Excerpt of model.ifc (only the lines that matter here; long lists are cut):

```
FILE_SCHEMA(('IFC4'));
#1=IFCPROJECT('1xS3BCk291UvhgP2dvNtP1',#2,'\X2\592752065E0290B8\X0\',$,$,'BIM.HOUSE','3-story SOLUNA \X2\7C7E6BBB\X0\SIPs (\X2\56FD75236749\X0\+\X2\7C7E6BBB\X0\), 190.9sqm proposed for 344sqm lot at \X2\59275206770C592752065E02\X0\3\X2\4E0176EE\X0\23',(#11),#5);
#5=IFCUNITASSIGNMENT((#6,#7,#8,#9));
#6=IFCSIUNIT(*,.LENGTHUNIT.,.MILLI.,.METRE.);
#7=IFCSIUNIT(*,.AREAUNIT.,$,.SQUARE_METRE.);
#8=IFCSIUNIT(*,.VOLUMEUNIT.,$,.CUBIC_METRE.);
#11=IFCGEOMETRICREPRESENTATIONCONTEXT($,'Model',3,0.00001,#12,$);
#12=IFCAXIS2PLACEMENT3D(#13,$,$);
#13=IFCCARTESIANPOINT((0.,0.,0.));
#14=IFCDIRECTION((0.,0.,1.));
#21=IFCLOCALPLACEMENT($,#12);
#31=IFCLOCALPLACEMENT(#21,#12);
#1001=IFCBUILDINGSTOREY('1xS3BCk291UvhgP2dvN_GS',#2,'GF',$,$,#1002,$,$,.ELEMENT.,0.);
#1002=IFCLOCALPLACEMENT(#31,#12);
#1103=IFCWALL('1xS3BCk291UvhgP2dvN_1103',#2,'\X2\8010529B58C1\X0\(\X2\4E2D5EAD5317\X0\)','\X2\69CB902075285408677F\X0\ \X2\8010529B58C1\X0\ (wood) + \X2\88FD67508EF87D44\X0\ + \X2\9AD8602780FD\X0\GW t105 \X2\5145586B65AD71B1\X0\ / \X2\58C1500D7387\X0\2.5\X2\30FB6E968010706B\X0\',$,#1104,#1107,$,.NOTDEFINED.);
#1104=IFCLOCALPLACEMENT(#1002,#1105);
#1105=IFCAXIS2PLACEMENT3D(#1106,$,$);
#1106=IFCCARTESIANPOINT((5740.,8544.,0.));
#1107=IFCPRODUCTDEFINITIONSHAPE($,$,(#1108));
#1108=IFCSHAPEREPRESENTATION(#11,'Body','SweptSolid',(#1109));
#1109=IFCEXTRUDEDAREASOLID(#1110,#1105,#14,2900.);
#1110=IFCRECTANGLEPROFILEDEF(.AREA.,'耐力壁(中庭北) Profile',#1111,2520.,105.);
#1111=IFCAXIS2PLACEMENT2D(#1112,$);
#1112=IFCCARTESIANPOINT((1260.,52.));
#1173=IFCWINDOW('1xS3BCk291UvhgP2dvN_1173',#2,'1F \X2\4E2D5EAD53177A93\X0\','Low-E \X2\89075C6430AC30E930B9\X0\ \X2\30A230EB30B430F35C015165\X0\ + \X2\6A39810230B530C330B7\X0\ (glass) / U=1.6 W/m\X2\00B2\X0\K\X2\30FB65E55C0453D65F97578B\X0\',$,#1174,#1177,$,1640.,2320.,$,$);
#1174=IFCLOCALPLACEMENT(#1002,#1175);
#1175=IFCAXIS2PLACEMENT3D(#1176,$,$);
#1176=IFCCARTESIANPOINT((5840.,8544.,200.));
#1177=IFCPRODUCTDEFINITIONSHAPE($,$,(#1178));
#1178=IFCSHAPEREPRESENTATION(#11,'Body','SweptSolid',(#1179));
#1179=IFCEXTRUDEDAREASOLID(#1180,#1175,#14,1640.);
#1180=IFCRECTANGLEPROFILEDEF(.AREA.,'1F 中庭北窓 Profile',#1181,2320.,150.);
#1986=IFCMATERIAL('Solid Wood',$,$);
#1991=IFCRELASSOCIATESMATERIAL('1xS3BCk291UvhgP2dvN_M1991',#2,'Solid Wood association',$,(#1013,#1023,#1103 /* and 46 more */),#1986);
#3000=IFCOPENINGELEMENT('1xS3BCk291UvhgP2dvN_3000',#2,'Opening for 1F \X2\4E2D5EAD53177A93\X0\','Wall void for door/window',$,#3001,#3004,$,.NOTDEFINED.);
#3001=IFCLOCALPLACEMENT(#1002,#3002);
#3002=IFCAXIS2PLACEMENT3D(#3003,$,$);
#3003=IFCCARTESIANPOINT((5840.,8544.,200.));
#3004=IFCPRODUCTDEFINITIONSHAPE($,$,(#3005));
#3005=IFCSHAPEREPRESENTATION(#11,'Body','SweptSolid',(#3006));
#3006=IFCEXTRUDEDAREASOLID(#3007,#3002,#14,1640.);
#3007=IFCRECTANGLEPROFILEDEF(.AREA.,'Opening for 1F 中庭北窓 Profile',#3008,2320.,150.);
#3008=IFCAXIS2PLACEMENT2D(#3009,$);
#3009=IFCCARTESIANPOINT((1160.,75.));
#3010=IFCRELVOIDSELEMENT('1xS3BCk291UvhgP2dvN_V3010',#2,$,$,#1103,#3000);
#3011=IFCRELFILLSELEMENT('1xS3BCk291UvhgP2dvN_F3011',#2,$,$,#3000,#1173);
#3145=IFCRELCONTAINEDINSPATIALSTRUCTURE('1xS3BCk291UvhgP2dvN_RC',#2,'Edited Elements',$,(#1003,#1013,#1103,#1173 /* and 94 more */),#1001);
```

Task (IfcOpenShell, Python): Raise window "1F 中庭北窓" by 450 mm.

```python
import numpy as np
import ifcopenshell
import ifcopenshell.api.geometry
import ifcopenshell.util.placement
import ifcopenshell.util.unit

model = ifcopenshell.open("model.ifc")
unit_scale = ifcopenshell.util.unit.calculate_unit_scale(model)

window = model.by_id(1173)
opening = window.FillsVoids[0].RelatingOpeningElement
dz = 450.0

shift = np.array([0.0, 0.0, dz])
# The window is not placed relative to its opening, so move both.
for product in (opening, window):
    matrix = ifcopenshell.util.placement.get_local_placement(product.ObjectPlacement)
    matrix[:3, 3] += shift
    ifcopenshell.api.geometry.edit_object_placement(model, product=product, matrix=matrix, is_si=False)

print(f"moved by {dz * unit_scale:+.3f} m")

model.write("model-out.ifc")
```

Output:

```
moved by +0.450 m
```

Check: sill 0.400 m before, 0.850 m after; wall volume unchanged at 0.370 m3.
